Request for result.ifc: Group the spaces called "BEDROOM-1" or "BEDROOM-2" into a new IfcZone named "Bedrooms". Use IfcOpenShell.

First a look at what the model holds.

```python
import ifcopenshell

model = ifcopenshell.open("result.ifc")
print(model.schema)
seen = {}
for space in model.by_type("IfcSpace"):
    seen[space.Name] = seen.get(space.Name, 0) + 1
for name, count in sorted(seen.items(), key=str):
    print(count, "x", name)
print("zones:", [z.Name for z in model.by_type("IfcZone")][:20])
```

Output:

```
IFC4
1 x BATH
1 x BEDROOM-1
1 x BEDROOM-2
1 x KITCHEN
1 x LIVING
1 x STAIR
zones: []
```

```python
import ifcopenshell
import ifcopenshell.api.group
import ifcopenshell.api.root

model = ifcopenshell.open("result.ifc")

names = {"BEDROOM-1", "BEDROOM-2"}
spaces = [s for s in model.by_type("IfcSpace") if s.Name in names]

zone = ifcopenshell.api.root.create_entity(model, ifc_class="IfcZone", name="Bedrooms")
ifcopenshell.api.group.assign_group(model, products=spaces, group=zone)
print(len(spaces), "spaces in", zone.Name)

model.write("result_rev.ifc")
```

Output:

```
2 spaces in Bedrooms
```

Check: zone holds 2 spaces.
